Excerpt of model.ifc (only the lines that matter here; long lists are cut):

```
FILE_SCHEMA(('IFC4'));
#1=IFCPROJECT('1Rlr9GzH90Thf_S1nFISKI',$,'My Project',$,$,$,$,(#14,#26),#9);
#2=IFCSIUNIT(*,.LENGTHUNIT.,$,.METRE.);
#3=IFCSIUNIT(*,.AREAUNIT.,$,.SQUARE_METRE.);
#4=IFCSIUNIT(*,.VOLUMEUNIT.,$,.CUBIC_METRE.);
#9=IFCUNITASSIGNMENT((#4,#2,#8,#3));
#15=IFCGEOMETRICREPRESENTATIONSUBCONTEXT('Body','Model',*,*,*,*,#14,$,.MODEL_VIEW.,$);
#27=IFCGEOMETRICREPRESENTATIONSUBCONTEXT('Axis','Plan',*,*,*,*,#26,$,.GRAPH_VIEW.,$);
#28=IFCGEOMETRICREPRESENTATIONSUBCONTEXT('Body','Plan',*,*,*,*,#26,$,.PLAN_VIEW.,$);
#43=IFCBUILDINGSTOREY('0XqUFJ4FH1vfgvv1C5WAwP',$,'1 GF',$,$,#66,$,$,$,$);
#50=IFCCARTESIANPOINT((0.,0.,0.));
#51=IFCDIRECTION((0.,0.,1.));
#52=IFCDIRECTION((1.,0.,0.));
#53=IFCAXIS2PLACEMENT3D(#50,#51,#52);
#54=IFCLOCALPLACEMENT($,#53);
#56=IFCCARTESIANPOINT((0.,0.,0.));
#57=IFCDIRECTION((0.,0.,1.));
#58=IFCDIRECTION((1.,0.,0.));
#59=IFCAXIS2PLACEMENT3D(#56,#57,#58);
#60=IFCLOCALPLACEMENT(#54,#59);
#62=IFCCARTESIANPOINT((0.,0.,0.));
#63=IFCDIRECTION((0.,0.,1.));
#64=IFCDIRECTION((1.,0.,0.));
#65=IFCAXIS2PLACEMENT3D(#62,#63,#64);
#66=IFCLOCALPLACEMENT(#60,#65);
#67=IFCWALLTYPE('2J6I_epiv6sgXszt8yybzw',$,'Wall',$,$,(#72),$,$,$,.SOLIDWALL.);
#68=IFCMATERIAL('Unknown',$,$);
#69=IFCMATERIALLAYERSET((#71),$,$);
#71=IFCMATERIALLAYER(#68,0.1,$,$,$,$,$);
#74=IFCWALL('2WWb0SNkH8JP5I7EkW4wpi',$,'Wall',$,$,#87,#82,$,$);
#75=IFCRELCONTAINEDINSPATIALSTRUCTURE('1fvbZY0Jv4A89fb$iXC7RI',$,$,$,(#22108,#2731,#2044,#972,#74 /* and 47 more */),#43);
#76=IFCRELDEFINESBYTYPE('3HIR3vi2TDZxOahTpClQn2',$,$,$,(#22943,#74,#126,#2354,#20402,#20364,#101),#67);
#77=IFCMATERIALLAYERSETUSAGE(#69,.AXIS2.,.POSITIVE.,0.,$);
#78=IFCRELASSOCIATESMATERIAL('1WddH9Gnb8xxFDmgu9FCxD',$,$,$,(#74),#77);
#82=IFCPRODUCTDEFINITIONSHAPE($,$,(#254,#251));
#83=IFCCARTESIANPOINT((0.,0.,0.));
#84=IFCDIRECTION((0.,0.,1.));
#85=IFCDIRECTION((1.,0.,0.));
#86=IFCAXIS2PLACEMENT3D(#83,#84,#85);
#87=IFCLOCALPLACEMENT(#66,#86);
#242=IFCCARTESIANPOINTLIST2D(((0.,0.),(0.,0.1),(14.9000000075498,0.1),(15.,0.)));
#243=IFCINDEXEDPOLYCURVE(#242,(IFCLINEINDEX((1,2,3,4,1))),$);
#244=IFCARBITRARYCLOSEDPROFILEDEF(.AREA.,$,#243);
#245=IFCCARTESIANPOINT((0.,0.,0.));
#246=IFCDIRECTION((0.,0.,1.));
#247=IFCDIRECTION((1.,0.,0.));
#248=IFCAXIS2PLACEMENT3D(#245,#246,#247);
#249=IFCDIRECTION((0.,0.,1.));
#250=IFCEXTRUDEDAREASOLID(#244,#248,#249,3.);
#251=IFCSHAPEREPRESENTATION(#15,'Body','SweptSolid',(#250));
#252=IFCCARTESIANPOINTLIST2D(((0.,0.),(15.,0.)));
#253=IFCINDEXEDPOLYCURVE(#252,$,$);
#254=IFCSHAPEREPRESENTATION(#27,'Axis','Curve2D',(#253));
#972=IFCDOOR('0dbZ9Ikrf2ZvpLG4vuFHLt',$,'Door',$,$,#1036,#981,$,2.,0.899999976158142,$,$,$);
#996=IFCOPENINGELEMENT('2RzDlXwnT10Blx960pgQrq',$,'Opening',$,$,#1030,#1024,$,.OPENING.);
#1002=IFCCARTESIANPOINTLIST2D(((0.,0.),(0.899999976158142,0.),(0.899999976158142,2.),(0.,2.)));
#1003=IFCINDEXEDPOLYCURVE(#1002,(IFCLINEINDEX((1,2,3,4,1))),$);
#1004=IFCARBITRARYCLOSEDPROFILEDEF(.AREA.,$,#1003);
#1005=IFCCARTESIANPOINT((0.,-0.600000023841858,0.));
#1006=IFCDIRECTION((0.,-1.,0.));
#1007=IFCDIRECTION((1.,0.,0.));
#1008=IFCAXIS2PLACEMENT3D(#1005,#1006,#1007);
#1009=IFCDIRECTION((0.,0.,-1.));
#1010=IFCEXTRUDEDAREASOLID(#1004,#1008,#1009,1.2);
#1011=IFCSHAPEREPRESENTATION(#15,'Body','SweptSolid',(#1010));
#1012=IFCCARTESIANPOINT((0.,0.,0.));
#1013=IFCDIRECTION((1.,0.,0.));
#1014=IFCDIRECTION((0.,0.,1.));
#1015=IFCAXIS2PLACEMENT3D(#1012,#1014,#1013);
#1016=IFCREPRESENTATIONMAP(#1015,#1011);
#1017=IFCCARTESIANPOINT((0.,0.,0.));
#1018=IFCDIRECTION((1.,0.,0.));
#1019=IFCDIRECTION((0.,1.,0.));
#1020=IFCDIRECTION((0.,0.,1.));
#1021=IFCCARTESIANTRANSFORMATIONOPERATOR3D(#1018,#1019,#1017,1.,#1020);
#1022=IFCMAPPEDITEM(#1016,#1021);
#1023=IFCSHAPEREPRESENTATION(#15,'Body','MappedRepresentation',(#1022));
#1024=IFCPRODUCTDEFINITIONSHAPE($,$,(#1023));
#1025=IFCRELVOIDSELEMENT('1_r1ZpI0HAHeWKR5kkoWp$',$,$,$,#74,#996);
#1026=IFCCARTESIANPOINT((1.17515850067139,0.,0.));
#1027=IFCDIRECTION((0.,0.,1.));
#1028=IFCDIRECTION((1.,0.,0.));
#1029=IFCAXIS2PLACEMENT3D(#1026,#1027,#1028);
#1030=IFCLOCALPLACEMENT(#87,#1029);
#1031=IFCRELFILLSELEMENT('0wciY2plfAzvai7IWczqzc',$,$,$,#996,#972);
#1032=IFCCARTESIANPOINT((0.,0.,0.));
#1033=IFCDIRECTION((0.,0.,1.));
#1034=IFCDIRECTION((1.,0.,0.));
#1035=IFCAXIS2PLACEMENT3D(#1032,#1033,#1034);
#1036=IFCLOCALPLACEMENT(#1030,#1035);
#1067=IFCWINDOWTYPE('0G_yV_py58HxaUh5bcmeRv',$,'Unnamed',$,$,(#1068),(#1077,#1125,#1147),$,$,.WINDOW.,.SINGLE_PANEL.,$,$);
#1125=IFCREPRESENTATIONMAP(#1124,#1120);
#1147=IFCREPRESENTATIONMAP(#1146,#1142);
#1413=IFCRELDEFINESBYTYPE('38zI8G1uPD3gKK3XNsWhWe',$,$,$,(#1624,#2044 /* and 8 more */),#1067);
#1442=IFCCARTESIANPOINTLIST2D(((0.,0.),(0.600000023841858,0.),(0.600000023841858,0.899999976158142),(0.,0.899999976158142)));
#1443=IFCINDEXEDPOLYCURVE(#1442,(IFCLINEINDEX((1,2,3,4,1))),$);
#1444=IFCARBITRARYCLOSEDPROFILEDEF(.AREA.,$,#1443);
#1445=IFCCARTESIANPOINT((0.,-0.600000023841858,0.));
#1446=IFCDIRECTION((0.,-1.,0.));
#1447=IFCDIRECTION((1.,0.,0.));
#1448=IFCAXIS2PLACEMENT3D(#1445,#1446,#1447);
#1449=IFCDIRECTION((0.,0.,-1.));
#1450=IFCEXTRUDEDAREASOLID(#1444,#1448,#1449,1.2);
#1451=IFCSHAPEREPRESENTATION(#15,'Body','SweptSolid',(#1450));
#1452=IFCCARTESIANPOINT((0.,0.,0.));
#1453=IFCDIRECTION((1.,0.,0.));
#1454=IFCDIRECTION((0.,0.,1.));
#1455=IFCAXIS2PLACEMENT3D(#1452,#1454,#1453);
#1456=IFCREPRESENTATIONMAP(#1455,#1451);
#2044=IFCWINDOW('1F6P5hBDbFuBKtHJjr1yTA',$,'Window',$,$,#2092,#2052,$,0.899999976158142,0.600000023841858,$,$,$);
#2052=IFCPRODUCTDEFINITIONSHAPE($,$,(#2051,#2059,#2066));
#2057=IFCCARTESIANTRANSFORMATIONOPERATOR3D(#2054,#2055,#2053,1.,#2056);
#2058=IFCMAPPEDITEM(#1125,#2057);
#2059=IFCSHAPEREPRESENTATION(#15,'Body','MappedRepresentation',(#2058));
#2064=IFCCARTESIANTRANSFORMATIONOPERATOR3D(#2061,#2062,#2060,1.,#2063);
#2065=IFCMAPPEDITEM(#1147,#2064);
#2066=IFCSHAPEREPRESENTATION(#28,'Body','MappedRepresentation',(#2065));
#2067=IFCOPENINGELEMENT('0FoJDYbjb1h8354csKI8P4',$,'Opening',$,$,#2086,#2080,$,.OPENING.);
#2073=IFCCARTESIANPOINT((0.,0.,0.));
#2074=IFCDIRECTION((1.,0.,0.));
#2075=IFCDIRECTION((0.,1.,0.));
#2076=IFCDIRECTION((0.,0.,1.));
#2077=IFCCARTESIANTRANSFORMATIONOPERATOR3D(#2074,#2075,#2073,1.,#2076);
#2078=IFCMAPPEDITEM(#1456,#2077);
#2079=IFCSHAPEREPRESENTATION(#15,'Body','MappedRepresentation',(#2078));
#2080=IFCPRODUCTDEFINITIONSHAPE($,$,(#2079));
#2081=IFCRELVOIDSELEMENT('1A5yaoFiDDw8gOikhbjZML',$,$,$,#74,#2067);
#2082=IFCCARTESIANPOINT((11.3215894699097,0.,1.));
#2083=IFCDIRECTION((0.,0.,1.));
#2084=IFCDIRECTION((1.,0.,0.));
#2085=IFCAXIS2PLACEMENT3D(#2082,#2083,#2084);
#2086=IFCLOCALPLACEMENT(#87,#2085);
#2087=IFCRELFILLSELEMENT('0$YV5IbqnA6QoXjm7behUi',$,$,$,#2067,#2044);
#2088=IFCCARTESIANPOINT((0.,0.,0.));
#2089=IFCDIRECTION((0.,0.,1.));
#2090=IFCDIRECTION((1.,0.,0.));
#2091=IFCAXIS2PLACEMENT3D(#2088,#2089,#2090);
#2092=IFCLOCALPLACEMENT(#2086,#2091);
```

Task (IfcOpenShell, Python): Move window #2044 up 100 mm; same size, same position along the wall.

```python
import numpy as np
import ifcopenshell
import ifcopenshell.api.geometry
import ifcopenshell.util.placement
import ifcopenshell.util.unit

model = ifcopenshell.open("model.ifc")
unit_scale = ifcopenshell.util.unit.calculate_unit_scale(model)

window = model.by_guid("1F6P5hBDbFuBKtHJjr1yTA")
opening = window.FillsVoids[0].RelatingOpeningElement
dz = 0.1

shift = np.array([0.0, 0.0, dz])
# The window is placed relative to its opening, so it follows when the opening moves.
matrix = ifcopenshell.util.placement.get_local_placement(opening.ObjectPlacement)
matrix[:3, 3] += shift
ifcopenshell.api.geometry.edit_object_placement(
    model, product=opening, matrix=matrix, is_si=False, should_transform_children=True
)

print(f"moved by {dz * unit_scale:+.3f} m")

model.write("model_rev.ifc")
```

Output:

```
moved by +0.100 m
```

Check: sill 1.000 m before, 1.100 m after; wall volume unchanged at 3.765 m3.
